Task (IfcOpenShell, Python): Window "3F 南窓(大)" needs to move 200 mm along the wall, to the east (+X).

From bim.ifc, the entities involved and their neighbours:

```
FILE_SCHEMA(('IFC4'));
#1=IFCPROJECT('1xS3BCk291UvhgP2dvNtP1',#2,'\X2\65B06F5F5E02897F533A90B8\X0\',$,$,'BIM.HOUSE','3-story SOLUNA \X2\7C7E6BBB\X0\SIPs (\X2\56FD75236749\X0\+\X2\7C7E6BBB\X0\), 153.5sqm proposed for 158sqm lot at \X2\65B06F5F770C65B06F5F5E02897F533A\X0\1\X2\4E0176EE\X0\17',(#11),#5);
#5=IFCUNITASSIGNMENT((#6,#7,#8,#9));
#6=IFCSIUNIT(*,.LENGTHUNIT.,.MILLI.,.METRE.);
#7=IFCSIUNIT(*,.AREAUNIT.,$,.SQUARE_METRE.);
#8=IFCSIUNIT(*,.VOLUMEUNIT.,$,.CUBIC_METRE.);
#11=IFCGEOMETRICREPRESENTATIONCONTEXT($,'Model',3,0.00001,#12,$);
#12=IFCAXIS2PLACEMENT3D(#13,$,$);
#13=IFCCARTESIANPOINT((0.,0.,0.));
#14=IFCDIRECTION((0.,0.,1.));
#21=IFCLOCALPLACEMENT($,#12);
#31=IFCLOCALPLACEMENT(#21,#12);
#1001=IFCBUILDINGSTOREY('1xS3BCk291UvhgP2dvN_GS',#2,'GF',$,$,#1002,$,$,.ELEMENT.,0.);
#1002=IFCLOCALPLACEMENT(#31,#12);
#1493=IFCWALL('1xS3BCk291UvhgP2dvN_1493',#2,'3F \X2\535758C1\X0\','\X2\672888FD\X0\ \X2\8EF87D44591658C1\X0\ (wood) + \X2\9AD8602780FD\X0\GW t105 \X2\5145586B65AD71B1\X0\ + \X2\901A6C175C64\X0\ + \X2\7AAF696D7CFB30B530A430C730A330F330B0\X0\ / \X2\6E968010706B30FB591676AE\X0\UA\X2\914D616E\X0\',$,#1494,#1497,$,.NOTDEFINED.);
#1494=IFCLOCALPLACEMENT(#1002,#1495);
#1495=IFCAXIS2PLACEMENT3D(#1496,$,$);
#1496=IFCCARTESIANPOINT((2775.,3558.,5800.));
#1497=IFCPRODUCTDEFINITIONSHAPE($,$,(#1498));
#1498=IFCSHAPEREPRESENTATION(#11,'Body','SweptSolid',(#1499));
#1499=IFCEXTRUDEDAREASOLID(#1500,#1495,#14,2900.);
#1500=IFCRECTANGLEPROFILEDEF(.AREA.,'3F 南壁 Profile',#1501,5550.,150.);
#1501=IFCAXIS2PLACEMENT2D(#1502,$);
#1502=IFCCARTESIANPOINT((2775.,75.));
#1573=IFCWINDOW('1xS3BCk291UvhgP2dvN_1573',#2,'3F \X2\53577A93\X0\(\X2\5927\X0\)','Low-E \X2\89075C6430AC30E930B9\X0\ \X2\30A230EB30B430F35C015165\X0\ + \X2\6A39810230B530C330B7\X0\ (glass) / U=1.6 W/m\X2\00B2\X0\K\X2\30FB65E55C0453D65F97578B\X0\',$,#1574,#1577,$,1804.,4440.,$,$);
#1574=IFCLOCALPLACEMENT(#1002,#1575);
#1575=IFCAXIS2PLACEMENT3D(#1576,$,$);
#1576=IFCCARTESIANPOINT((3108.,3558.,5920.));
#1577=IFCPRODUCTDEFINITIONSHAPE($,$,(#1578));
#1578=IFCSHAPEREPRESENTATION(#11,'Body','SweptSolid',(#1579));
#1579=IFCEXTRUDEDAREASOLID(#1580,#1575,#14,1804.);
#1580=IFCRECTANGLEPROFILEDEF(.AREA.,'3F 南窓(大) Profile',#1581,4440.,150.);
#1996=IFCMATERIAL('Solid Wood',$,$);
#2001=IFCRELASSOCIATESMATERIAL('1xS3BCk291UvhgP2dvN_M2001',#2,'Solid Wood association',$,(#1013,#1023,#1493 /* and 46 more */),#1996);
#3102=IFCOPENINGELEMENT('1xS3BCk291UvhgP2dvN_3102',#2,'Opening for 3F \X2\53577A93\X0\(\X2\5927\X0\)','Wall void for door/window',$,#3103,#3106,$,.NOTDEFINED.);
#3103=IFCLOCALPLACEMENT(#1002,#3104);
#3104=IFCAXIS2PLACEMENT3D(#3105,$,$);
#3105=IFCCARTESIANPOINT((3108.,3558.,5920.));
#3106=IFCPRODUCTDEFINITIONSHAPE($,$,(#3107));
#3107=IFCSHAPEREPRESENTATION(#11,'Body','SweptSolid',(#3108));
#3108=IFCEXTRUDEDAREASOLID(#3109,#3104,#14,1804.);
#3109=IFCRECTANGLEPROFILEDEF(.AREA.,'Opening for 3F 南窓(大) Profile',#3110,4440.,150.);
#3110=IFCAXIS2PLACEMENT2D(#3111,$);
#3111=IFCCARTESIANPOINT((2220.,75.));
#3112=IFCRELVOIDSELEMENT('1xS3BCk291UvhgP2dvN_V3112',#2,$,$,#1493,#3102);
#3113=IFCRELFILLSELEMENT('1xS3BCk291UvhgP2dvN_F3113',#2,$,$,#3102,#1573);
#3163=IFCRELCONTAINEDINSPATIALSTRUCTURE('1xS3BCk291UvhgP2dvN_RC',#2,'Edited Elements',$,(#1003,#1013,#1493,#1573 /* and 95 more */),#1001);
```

```python
import ifcopenshell
import ifcopenshell.api.geometry
import ifcopenshell.util.placement
import ifcopenshell.util.unit

model = ifcopenshell.open("bim.ifc")
unit_scale = ifcopenshell.util.unit.calculate_unit_scale(model)

window = model.by_id(1573)
opening = window.FillsVoids[0].RelatingOpeningElement
wall = opening.VoidsElements[0].RelatingBuildingElement

wall_matrix = ifcopenshell.util.placement.get_local_placement(wall.ObjectPlacement)
shift = wall_matrix[:3, 0] * 0.2 / unit_scale
before = ifcopenshell.util.placement.get_local_placement(window.ObjectPlacement)[:3, 3].copy()

# The window is not placed relative to its opening, so move both.
for product in (opening, window):
    matrix = ifcopenshell.util.placement.get_local_placement(product.ObjectPlacement)
    matrix[:3, 3] += shift
    ifcopenshell.api.geometry.edit_object_placement(model, product=product, matrix=matrix, is_si=False)

after = ifcopenshell.util.placement.get_local_placement(window.ObjectPlacement)[:3, 3]
print("window moved by", (after - before).round(3) + 0.0)

model.write("bim_rev.ifc")
```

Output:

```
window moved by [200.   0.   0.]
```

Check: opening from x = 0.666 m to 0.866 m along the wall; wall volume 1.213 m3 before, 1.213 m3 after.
